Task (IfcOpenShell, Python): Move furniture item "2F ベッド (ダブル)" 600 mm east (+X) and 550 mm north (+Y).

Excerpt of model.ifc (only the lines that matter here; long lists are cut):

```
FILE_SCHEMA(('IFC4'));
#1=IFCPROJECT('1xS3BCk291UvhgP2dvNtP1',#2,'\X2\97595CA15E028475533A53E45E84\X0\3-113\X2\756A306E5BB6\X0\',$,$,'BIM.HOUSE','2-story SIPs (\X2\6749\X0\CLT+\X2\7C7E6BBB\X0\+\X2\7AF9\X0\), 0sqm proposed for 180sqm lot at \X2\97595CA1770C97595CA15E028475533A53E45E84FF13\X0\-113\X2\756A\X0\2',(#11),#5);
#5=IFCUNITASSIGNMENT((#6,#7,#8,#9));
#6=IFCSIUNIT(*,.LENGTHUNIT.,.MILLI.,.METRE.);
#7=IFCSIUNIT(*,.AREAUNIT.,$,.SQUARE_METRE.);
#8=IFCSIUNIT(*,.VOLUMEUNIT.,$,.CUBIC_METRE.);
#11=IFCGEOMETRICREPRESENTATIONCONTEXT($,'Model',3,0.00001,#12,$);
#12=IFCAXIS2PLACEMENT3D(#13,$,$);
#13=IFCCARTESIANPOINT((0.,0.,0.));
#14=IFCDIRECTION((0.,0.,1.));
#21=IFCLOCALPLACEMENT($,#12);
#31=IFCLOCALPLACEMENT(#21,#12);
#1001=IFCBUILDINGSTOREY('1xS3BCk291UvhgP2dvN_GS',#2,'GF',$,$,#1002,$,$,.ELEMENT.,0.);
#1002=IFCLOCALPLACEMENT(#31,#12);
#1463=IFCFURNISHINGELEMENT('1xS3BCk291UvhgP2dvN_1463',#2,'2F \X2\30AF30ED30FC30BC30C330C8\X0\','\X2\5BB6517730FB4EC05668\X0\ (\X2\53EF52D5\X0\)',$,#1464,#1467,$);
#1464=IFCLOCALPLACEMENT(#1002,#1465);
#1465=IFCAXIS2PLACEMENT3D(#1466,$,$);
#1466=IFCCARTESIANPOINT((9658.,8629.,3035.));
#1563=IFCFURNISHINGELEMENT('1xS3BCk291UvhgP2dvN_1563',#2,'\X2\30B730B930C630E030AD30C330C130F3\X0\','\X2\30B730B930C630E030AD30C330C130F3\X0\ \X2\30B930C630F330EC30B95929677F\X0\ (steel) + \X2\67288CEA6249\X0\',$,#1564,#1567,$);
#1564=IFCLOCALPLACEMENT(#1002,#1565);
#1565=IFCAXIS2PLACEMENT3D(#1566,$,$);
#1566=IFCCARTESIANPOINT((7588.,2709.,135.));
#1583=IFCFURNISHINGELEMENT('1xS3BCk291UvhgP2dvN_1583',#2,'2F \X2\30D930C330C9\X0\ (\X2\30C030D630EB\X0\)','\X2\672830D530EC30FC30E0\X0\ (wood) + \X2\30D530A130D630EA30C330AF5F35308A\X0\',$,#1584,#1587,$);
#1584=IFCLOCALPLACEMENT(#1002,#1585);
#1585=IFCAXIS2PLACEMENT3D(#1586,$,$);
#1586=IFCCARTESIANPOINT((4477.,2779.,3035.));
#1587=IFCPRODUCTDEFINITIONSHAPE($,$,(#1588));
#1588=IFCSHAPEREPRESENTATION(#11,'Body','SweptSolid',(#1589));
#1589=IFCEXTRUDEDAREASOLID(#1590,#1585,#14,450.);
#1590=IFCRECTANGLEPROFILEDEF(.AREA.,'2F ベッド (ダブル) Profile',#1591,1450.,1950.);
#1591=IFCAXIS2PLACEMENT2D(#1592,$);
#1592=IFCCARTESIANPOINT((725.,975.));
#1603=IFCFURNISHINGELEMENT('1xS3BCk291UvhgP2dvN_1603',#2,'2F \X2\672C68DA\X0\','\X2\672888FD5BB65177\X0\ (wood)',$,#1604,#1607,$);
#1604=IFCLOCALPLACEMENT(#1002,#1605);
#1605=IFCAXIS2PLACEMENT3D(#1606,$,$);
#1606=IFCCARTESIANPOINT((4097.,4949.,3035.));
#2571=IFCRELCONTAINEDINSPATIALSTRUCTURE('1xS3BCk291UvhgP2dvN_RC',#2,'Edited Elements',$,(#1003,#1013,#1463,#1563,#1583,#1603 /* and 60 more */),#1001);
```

```python
import ifcopenshell
import ifcopenshell.api.geometry
import ifcopenshell.util.placement

model = ifcopenshell.open("model.ifc")

item = model.by_id(1583)
matrix = ifcopenshell.util.placement.get_local_placement(item.ObjectPlacement)
matrix[0, 3] += 600.0
matrix[1, 3] += 550.0
ifcopenshell.api.geometry.edit_object_placement(model, product=item, matrix=matrix, is_si=False)

print(ifcopenshell.util.placement.get_local_placement(item.ObjectPlacement).round(3) + 0.0)

model.write("model-out.ifc")
```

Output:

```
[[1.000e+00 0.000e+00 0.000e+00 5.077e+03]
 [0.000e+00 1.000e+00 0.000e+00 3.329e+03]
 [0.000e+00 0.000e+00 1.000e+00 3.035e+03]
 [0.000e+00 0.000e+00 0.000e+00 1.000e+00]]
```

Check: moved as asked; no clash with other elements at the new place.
